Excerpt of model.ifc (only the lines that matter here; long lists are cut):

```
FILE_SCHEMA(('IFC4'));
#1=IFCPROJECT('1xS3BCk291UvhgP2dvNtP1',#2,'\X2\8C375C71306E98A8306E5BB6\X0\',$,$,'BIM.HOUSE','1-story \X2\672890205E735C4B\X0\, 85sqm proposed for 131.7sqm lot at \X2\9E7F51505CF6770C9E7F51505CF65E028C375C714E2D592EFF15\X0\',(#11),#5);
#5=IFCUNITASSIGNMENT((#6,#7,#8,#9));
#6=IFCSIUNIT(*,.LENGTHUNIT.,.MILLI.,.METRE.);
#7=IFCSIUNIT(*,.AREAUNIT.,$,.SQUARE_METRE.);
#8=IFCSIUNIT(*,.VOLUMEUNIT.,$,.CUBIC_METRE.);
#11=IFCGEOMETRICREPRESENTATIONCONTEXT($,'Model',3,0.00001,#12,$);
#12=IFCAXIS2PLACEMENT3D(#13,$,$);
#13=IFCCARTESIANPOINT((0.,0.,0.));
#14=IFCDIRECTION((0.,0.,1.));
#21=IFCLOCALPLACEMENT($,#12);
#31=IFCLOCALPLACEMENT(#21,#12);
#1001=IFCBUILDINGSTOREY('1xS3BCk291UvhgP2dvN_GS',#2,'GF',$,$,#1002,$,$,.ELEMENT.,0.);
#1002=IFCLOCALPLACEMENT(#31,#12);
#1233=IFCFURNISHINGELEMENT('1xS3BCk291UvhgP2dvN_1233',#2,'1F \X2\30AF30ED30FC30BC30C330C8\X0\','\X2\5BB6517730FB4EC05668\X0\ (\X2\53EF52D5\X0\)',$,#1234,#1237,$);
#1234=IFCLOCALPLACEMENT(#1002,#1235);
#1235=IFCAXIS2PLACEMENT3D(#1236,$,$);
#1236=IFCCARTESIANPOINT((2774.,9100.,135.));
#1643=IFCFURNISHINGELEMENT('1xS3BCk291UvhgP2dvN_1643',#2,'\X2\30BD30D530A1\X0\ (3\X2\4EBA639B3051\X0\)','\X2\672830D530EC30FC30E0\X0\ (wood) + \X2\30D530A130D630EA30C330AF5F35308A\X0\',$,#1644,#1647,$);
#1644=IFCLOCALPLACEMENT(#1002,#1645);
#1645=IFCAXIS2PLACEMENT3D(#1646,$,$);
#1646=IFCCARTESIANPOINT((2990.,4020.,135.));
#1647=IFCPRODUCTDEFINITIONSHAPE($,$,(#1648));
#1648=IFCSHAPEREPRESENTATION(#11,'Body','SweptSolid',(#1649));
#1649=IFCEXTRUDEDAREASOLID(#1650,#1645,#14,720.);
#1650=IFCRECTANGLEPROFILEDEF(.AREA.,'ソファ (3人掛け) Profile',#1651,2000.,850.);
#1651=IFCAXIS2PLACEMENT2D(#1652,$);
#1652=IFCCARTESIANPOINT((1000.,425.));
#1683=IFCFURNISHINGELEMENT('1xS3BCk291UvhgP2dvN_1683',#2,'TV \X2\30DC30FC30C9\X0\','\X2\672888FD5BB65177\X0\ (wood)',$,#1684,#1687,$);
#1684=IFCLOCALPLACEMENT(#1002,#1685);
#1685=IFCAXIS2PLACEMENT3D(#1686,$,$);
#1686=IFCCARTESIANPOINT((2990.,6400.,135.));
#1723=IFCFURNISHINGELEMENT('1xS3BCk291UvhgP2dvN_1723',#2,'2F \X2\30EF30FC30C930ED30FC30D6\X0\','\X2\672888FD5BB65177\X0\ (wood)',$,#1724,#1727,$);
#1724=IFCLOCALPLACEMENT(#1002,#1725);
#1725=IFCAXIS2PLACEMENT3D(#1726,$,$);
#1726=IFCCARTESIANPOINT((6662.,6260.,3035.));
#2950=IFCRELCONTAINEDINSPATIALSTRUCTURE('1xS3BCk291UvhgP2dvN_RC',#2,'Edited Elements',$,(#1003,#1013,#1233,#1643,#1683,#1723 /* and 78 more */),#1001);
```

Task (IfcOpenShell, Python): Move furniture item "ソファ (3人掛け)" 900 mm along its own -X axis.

```python
import ifcopenshell
import ifcopenshell.api.geometry
import ifcopenshell.util.placement

model = ifcopenshell.open("model.ifc")

item = model.by_guid("1xS3BCk291UvhgP2dvN_1643")
matrix = ifcopenshell.util.placement.get_local_placement(item.ObjectPlacement)
matrix[:3, 3] -= matrix[:3, 0] * 900.0
ifcopenshell.api.geometry.edit_object_placement(model, product=item, matrix=matrix, is_si=False)

print(ifcopenshell.util.placement.get_local_placement(item.ObjectPlacement).round(3) + 0.0)

model.write("model-out.ifc")
```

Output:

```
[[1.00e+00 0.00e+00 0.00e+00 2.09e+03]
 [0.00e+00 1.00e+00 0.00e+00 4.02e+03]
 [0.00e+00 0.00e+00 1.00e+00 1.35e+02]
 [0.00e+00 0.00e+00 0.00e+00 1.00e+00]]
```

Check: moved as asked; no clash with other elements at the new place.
